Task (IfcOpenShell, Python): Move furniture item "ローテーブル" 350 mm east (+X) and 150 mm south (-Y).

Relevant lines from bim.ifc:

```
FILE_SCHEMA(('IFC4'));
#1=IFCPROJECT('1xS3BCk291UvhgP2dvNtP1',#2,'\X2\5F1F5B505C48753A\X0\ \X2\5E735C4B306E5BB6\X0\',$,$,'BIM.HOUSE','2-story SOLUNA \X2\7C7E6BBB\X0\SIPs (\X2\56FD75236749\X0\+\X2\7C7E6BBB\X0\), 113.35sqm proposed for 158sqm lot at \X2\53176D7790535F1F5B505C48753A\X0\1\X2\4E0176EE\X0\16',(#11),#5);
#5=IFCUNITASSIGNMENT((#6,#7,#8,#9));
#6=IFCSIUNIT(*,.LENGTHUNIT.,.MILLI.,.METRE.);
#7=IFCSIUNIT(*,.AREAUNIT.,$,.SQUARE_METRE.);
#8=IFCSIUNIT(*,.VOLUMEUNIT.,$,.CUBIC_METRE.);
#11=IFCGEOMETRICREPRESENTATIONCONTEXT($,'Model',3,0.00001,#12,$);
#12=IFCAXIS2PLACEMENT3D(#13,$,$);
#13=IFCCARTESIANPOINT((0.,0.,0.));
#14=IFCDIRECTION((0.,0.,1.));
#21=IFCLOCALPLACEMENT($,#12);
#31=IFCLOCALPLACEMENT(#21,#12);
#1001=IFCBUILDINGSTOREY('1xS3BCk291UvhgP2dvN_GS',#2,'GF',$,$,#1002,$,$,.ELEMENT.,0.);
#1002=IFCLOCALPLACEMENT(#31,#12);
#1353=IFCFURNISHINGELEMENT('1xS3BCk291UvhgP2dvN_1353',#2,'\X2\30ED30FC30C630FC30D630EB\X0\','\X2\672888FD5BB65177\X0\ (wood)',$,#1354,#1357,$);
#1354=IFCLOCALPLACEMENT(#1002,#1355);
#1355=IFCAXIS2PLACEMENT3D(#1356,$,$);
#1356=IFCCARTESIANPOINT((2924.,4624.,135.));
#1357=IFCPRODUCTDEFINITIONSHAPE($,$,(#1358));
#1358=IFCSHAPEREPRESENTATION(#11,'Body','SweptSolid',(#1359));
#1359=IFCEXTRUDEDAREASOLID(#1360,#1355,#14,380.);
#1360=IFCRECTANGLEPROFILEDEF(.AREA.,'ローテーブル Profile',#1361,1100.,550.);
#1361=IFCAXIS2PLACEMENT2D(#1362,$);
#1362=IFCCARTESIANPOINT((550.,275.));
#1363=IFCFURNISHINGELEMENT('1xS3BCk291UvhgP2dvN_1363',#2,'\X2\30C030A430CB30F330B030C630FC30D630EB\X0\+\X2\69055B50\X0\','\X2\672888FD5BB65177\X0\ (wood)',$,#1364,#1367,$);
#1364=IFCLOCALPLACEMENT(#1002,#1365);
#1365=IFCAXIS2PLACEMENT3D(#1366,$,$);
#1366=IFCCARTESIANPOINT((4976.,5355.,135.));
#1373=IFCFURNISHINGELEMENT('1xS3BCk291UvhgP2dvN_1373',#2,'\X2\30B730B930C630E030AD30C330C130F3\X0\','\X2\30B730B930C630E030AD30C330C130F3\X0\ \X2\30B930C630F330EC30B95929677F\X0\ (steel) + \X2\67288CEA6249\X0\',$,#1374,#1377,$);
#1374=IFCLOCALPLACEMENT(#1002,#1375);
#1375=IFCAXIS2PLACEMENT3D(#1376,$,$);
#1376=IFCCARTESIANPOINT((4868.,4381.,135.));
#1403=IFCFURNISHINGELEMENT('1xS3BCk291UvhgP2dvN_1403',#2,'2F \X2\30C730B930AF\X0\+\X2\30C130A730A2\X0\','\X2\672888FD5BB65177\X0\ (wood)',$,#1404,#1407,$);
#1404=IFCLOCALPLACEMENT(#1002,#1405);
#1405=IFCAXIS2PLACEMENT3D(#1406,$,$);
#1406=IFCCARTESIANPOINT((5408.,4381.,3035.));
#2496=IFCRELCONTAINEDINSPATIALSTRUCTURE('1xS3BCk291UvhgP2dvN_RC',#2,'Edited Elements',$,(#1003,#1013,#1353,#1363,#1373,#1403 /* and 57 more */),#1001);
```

```python
import ifcopenshell
import ifcopenshell.api.geometry
import ifcopenshell.util.placement
import ifcopenshell.util.unit

model = ifcopenshell.open("bim.ifc")
unit_scale = ifcopenshell.util.unit.calculate_unit_scale(model)

item = model.by_id(1353)
matrix = ifcopenshell.util.placement.get_local_placement(item.ObjectPlacement)
matrix[0, 3] += 0.35 / unit_scale
matrix[1, 3] -= 0.15 / unit_scale
ifcopenshell.api.geometry.edit_object_placement(model, product=item, matrix=matrix, is_si=False)

print(ifcopenshell.util.placement.get_local_placement(item.ObjectPlacement).round(3) + 0.0)

model.write("bim_edited.ifc")
```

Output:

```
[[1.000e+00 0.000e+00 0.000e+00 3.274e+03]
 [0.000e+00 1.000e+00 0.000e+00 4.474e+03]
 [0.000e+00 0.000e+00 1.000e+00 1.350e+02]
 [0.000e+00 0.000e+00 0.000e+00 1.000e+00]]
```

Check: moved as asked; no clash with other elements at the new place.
